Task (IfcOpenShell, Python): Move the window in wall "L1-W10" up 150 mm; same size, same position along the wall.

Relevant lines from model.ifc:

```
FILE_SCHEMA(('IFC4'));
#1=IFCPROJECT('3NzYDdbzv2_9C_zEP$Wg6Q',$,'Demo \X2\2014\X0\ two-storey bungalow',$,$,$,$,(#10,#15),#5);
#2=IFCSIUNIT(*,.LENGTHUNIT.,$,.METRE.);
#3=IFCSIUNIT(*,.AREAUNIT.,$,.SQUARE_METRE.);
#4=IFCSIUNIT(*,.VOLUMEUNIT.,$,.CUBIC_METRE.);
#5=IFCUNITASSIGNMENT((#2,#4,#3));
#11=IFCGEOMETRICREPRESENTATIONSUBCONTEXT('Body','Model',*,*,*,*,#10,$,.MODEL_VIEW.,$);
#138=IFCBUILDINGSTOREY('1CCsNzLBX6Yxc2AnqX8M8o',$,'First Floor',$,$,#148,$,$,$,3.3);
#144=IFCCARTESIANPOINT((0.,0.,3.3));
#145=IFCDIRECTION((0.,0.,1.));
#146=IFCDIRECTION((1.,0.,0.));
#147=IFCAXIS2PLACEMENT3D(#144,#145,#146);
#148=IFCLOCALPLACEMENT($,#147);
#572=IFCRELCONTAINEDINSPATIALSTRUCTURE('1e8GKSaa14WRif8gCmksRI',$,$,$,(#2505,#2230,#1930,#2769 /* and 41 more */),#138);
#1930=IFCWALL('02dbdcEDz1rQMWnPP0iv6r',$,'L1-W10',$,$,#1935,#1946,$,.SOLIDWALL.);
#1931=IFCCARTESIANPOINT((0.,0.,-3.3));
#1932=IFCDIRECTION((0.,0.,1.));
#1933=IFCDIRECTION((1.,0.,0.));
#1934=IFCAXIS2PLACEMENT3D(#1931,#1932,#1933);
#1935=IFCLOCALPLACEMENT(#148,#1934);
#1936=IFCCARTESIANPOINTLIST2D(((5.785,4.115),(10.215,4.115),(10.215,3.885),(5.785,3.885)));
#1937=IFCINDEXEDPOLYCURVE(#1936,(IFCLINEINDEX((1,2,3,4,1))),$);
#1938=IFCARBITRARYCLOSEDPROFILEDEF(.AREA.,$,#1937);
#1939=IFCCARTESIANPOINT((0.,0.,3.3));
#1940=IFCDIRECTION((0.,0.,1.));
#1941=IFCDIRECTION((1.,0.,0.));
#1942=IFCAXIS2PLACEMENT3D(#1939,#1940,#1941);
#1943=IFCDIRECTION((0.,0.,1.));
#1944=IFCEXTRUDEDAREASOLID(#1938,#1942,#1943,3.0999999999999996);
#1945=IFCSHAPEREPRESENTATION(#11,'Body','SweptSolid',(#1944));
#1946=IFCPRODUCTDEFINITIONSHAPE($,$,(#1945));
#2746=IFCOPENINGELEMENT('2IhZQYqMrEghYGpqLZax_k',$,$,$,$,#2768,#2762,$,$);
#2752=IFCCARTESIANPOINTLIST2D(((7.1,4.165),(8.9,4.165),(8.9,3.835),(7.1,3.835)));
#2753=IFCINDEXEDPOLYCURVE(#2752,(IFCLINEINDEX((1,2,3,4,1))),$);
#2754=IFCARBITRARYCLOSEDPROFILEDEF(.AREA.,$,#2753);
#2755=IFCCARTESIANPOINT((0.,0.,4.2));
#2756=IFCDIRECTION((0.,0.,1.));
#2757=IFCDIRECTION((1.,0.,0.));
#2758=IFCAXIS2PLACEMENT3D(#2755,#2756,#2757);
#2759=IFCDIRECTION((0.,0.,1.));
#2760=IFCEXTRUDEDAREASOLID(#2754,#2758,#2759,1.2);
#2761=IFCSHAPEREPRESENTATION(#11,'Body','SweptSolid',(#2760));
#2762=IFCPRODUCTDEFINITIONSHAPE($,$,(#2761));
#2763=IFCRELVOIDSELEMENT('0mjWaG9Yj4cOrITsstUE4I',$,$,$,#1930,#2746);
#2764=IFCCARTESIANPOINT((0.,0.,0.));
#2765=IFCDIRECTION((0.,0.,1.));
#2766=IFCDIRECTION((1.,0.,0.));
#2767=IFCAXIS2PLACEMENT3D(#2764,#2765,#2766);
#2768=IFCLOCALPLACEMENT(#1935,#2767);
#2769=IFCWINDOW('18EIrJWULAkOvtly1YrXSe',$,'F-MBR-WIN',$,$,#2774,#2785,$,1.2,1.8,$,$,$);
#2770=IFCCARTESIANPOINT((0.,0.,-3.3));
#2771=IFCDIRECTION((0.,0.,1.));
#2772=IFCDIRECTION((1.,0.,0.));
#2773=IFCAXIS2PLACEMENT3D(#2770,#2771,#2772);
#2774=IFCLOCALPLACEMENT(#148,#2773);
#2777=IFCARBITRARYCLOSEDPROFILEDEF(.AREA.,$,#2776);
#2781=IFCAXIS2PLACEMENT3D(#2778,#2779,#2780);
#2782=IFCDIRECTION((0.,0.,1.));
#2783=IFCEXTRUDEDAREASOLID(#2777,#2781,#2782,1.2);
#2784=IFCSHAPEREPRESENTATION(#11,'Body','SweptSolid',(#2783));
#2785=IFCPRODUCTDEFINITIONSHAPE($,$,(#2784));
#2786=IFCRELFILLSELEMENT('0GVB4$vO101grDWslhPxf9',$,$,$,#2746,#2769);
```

```python
import numpy as np
import ifcopenshell
import ifcopenshell.api.geometry
import ifcopenshell.util.placement
import ifcopenshell.util.unit

model = ifcopenshell.open("model.ifc")
unit_scale = ifcopenshell.util.unit.calculate_unit_scale(model)

window = model.by_guid("18EIrJWULAkOvtly1YrXSe")
opening = window.FillsVoids[0].RelatingOpeningElement
dz = 0.15

shift = np.array([0.0, 0.0, dz])
# The window is not placed relative to its opening, so move both.
for product in (opening, window):
    matrix = ifcopenshell.util.placement.get_local_placement(product.ObjectPlacement)
    matrix[:3, 3] += shift
    ifcopenshell.api.geometry.edit_object_placement(model, product=product, matrix=matrix, is_si=False)

print(f"moved by {dz * unit_scale:+.3f} m")

model.write("model_updated.ifc")
```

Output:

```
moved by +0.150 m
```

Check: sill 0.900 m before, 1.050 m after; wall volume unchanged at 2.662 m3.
